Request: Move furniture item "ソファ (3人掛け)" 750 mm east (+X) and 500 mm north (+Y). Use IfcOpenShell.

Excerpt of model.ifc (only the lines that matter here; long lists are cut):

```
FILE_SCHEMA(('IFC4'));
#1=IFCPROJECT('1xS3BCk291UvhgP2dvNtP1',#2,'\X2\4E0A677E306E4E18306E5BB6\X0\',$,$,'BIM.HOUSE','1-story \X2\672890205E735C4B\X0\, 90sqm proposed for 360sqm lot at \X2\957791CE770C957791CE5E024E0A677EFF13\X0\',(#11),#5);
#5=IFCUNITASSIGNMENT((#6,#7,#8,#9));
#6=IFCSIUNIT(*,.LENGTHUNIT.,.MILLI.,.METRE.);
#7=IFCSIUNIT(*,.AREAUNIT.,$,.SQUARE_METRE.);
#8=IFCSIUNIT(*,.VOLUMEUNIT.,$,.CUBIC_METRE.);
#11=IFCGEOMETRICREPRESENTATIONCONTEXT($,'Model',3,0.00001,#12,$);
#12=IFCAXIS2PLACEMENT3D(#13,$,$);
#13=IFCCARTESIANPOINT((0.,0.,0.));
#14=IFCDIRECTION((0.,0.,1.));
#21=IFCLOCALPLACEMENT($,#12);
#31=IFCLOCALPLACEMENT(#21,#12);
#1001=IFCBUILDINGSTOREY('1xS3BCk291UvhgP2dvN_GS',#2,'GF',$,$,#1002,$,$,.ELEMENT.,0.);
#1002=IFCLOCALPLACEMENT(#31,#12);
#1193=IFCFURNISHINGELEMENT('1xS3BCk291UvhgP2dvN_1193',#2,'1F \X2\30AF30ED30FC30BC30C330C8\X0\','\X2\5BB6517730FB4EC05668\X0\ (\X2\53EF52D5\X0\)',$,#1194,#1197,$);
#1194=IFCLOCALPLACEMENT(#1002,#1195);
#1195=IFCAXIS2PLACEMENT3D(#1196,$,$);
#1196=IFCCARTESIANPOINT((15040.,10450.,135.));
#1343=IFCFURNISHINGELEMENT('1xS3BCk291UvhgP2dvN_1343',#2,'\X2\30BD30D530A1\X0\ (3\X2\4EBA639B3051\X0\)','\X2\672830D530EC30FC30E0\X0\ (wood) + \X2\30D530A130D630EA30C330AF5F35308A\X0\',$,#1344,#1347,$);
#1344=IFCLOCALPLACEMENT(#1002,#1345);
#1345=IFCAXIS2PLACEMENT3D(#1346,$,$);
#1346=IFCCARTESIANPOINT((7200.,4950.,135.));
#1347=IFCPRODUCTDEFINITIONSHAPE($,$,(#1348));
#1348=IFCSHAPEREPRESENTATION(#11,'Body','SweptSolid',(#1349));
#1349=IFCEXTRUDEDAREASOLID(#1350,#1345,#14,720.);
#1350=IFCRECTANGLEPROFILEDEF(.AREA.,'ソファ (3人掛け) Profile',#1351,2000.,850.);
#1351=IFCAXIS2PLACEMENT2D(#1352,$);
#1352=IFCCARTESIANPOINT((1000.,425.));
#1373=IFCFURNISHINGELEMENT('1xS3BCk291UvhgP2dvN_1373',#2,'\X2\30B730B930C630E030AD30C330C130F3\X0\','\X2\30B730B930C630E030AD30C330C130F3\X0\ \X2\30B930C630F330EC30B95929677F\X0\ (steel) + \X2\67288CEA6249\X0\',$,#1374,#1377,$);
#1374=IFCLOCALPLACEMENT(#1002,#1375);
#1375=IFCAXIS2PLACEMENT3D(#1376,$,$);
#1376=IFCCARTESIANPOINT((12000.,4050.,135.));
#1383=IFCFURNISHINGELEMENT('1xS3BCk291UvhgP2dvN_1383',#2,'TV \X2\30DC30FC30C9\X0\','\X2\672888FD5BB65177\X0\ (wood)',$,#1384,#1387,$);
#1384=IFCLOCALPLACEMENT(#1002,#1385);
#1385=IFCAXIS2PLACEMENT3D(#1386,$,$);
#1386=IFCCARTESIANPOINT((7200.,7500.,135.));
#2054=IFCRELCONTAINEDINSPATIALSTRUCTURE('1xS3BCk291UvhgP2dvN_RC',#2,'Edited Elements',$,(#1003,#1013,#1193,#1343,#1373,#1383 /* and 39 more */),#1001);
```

```python
import ifcopenshell
import ifcopenshell.api.geometry
import ifcopenshell.util.placement
import ifcopenshell.util.unit

model = ifcopenshell.open("model.ifc")
unit_scale = ifcopenshell.util.unit.calculate_unit_scale(model)

item = model.by_guid("1xS3BCk291UvhgP2dvN_1343")
matrix = ifcopenshell.util.placement.get_local_placement(item.ObjectPlacement)
matrix[0, 3] += 0.75 / unit_scale
matrix[1, 3] += 0.5 / unit_scale
ifcopenshell.api.geometry.edit_object_placement(model, product=item, matrix=matrix, is_si=False)

print(ifcopenshell.util.placement.get_local_placement(item.ObjectPlacement).round(3) + 0.0)

model.write("model_v2.ifc")
```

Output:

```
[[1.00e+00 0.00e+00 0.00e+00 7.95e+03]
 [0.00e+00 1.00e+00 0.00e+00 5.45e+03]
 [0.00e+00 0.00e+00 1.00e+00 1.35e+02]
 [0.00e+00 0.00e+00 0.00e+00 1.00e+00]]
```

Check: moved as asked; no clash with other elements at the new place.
